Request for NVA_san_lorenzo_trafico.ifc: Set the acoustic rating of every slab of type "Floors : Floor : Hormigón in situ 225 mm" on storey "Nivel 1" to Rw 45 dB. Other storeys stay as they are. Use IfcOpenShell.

First a look at what the model holds.

```python
import ifcopenshell
import ifcopenshell.util.element

model = ifcopenshell.open("NVA_san_lorenzo_trafico.ifc")
print(model.schema)
storey = next(s for s in model.by_type("IfcBuildingStorey") if s.Name == "Nivel 1")
slabs = [e for e in ifcopenshell.util.element.get_decomposition(storey) if e.is_a("IfcSlab")]
seen = {}
for e in slabs:
    element_type = ifcopenshell.util.element.get_type(e)
    key = (element_type.Name if element_type != e and element_type else None, ifcopenshell.util.element.get_pset(e, "Pset_SlabCommon", "AcousticRating"))
    seen[key] = seen.get(key, 0) + 1
for (name, value), count in sorted(seen.items(), key=str):
    print(count, "x", name, "|", value)
```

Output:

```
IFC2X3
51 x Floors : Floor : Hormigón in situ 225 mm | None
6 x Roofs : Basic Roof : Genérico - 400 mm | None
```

```python
import ifcopenshell
import ifcopenshell.api.pset
import ifcopenshell.util.element

model = ifcopenshell.open("NVA_san_lorenzo_trafico.ifc")

storey = next(s for s in model.by_type("IfcBuildingStorey") if s.Name == "Nivel 1")
slabs = [e for e in ifcopenshell.util.element.get_decomposition(storey) if e.is_a("IfcSlab")]

count = 0
for e in slabs:
    element_type = ifcopenshell.util.element.get_type(e)
    if element_type in (None, e) or element_type.Name != "Floors : Floor : Hormigón in situ 225 mm":
        continue
    # add_pset returns the element's existing set when there is one.
    pset = ifcopenshell.api.pset.add_pset(model, product=e, name="Pset_SlabCommon")
    ifcopenshell.api.pset.edit_pset(model, pset=pset, properties={"AcousticRating": "Rw 45 dB"})
    count += 1

print(count, "slabs updated")

model.write("NVA_san_lorenzo_trafico_edited.ifc")
```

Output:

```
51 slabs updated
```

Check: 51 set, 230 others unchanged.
